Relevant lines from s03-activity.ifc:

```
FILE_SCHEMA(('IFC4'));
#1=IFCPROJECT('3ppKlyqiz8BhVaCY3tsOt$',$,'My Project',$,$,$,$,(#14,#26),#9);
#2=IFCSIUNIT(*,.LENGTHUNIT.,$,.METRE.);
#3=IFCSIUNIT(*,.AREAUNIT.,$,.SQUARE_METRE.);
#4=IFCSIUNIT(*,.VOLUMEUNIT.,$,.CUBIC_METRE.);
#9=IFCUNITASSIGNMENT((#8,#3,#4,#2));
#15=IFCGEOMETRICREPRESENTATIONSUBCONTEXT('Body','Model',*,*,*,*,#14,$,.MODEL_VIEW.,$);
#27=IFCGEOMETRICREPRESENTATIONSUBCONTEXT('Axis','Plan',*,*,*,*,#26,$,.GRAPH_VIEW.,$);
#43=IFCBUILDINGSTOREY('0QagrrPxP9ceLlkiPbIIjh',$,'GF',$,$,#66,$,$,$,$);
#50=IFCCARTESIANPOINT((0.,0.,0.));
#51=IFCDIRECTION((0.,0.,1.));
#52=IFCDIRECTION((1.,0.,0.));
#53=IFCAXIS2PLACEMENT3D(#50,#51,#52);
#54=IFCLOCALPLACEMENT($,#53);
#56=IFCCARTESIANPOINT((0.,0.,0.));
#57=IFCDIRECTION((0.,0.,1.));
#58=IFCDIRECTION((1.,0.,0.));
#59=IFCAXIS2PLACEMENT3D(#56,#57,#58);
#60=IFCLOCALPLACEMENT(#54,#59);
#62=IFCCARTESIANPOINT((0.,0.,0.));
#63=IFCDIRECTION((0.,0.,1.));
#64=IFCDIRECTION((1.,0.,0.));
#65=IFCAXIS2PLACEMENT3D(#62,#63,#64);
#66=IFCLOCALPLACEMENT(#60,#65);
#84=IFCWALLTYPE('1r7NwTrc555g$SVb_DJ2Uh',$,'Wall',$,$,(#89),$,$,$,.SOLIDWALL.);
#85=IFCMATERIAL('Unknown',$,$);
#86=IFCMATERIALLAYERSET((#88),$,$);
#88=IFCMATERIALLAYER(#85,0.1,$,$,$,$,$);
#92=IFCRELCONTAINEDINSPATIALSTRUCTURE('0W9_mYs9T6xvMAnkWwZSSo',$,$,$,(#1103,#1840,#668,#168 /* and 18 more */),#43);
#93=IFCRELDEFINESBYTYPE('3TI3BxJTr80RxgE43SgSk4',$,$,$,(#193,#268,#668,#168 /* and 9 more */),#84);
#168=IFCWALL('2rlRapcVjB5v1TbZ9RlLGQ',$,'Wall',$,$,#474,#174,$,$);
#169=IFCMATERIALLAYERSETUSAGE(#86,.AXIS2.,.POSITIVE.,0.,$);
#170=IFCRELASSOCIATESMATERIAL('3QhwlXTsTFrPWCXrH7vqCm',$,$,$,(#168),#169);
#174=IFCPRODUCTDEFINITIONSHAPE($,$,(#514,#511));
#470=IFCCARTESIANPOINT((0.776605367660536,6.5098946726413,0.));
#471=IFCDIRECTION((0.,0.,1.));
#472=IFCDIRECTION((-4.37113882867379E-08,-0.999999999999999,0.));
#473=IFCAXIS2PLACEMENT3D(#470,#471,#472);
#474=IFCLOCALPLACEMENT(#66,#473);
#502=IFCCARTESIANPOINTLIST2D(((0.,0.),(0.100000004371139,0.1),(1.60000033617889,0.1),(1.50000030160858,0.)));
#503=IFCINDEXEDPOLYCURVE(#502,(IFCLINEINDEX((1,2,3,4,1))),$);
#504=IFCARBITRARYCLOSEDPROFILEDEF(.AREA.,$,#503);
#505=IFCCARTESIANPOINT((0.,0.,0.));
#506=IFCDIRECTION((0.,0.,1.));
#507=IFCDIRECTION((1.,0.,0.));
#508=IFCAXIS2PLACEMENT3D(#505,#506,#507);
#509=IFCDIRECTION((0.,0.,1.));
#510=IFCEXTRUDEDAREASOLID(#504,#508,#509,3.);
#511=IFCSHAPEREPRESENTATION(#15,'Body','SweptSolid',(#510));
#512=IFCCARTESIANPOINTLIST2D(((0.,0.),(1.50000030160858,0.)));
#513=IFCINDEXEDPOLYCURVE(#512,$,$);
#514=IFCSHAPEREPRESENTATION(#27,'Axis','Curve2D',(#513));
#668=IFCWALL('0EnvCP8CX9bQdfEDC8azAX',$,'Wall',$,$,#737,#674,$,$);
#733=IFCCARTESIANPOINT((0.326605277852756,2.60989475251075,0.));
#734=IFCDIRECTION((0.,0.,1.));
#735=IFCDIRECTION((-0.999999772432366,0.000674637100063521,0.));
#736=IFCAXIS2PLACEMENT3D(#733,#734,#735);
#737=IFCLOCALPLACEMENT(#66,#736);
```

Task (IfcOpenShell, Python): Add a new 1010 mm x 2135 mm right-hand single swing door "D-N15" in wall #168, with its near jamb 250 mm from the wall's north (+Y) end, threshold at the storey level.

```python
import numpy as np
import ifcopenshell
import ifcopenshell.api.feature
import ifcopenshell.api.geometry
import ifcopenshell.api.root
import ifcopenshell.api.spatial
import ifcopenshell.geom
import ifcopenshell.util.element
import ifcopenshell.util.placement
import ifcopenshell.util.representation
import ifcopenshell.util.shape
import ifcopenshell.util.unit

model = ifcopenshell.open("s03-activity.ifc")
unit_scale = ifcopenshell.util.unit.calculate_unit_scale(model)
settings = ifcopenshell.geom.settings()


def volume(element):
    """Net volume in cubic metres, openings subtracted."""
    shape = ifcopenshell.geom.create_shape(settings, element)
    return ifcopenshell.util.shape.get_volume(shape.geometry)


wall = model.by_guid("2rlRapcVjB5v1TbZ9RlLGQ")
storey = ifcopenshell.util.element.get_container(wall, ifc_class="IfcBuildingStorey")
context = ifcopenshell.util.representation.get_context(model, "Model", "Body", "MODEL_VIEW")
before = volume(wall)

width, height, from_end, sill = 1.01, 2.135, 0.25, 0.0  # metres

# The wall runs along its own X axis, and the end named is its -X end.
wall_shape = ifcopenshell.geom.create_shape(settings, wall)
x, y, z = ifcopenshell.util.shape.get_vertices(wall_shape.geometry).T
start = x.min() + from_end
face, thickness = float(y.min()), float(y.max() - y.min())
wall_matrix = ifcopenshell.util.placement.get_local_placement(wall.ObjectPlacement)
level = ifcopenshell.util.placement.get_local_placement(storey.ObjectPlacement)[2, 3]


def in_wall(x, y):
    """Placement at x, y metres in the wall's axes, at sill height."""
    matrix = wall_matrix.copy()
    matrix[:, 3] = wall_matrix @ np.array([x / unit_scale, y / unit_scale, 0.0, 1.0])
    matrix[2, 3] = level + sill / unit_scale
    return matrix


# Opening: a box that overshoots both wall faces by 50 mm.
opening = ifcopenshell.api.root.create_entity(model, ifc_class="IfcOpeningElement", predefined_type="OPENING")
box = ifcopenshell.api.geometry.add_wall_representation(
    model, context=context, length=width, height=height, thickness=thickness + 0.1
)
ifcopenshell.api.geometry.assign_representation(model, product=opening, representation=box)
ifcopenshell.api.geometry.edit_object_placement(model, product=opening, matrix=in_wall(start, face - 0.05), is_si=False)
ifcopenshell.api.feature.add_feature(model, feature=opening, element=wall)

door = ifcopenshell.api.root.create_entity(model, ifc_class="IfcDoor", name="D-N15", predefined_type="DOOR")
door.OverallWidth, door.OverallHeight = width / unit_scale, height / unit_scale
door.OperationType = "SINGLE_SWING_RIGHT"
body = ifcopenshell.api.geometry.add_door_representation(
    model,
    context=context,
    overall_width=door.OverallWidth,
    overall_height=door.OverallHeight,
    operation_type="SINGLE_SWING_RIGHT",
    lining_properties={"LiningDepth": thickness / unit_scale, "ThresholdDepth": thickness / unit_scale},
)
ifcopenshell.api.geometry.assign_representation(model, product=door, representation=body)
ifcopenshell.api.spatial.assign_container(model, products=[door], relating_structure=storey)
ifcopenshell.api.feature.add_filling(model, opening=opening, element=door)

# The lining spans the wall, so the door starts at the wall face.
ifcopenshell.api.geometry.edit_object_placement(model, product=door, matrix=in_wall(start, face), is_si=False)

after = volume(wall)

print(f"wall volume {before:.3f} -> {after:.3f} m3")

model.write("s03-activity_v2.ifc")
```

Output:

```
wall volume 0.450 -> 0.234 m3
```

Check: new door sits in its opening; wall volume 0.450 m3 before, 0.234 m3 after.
